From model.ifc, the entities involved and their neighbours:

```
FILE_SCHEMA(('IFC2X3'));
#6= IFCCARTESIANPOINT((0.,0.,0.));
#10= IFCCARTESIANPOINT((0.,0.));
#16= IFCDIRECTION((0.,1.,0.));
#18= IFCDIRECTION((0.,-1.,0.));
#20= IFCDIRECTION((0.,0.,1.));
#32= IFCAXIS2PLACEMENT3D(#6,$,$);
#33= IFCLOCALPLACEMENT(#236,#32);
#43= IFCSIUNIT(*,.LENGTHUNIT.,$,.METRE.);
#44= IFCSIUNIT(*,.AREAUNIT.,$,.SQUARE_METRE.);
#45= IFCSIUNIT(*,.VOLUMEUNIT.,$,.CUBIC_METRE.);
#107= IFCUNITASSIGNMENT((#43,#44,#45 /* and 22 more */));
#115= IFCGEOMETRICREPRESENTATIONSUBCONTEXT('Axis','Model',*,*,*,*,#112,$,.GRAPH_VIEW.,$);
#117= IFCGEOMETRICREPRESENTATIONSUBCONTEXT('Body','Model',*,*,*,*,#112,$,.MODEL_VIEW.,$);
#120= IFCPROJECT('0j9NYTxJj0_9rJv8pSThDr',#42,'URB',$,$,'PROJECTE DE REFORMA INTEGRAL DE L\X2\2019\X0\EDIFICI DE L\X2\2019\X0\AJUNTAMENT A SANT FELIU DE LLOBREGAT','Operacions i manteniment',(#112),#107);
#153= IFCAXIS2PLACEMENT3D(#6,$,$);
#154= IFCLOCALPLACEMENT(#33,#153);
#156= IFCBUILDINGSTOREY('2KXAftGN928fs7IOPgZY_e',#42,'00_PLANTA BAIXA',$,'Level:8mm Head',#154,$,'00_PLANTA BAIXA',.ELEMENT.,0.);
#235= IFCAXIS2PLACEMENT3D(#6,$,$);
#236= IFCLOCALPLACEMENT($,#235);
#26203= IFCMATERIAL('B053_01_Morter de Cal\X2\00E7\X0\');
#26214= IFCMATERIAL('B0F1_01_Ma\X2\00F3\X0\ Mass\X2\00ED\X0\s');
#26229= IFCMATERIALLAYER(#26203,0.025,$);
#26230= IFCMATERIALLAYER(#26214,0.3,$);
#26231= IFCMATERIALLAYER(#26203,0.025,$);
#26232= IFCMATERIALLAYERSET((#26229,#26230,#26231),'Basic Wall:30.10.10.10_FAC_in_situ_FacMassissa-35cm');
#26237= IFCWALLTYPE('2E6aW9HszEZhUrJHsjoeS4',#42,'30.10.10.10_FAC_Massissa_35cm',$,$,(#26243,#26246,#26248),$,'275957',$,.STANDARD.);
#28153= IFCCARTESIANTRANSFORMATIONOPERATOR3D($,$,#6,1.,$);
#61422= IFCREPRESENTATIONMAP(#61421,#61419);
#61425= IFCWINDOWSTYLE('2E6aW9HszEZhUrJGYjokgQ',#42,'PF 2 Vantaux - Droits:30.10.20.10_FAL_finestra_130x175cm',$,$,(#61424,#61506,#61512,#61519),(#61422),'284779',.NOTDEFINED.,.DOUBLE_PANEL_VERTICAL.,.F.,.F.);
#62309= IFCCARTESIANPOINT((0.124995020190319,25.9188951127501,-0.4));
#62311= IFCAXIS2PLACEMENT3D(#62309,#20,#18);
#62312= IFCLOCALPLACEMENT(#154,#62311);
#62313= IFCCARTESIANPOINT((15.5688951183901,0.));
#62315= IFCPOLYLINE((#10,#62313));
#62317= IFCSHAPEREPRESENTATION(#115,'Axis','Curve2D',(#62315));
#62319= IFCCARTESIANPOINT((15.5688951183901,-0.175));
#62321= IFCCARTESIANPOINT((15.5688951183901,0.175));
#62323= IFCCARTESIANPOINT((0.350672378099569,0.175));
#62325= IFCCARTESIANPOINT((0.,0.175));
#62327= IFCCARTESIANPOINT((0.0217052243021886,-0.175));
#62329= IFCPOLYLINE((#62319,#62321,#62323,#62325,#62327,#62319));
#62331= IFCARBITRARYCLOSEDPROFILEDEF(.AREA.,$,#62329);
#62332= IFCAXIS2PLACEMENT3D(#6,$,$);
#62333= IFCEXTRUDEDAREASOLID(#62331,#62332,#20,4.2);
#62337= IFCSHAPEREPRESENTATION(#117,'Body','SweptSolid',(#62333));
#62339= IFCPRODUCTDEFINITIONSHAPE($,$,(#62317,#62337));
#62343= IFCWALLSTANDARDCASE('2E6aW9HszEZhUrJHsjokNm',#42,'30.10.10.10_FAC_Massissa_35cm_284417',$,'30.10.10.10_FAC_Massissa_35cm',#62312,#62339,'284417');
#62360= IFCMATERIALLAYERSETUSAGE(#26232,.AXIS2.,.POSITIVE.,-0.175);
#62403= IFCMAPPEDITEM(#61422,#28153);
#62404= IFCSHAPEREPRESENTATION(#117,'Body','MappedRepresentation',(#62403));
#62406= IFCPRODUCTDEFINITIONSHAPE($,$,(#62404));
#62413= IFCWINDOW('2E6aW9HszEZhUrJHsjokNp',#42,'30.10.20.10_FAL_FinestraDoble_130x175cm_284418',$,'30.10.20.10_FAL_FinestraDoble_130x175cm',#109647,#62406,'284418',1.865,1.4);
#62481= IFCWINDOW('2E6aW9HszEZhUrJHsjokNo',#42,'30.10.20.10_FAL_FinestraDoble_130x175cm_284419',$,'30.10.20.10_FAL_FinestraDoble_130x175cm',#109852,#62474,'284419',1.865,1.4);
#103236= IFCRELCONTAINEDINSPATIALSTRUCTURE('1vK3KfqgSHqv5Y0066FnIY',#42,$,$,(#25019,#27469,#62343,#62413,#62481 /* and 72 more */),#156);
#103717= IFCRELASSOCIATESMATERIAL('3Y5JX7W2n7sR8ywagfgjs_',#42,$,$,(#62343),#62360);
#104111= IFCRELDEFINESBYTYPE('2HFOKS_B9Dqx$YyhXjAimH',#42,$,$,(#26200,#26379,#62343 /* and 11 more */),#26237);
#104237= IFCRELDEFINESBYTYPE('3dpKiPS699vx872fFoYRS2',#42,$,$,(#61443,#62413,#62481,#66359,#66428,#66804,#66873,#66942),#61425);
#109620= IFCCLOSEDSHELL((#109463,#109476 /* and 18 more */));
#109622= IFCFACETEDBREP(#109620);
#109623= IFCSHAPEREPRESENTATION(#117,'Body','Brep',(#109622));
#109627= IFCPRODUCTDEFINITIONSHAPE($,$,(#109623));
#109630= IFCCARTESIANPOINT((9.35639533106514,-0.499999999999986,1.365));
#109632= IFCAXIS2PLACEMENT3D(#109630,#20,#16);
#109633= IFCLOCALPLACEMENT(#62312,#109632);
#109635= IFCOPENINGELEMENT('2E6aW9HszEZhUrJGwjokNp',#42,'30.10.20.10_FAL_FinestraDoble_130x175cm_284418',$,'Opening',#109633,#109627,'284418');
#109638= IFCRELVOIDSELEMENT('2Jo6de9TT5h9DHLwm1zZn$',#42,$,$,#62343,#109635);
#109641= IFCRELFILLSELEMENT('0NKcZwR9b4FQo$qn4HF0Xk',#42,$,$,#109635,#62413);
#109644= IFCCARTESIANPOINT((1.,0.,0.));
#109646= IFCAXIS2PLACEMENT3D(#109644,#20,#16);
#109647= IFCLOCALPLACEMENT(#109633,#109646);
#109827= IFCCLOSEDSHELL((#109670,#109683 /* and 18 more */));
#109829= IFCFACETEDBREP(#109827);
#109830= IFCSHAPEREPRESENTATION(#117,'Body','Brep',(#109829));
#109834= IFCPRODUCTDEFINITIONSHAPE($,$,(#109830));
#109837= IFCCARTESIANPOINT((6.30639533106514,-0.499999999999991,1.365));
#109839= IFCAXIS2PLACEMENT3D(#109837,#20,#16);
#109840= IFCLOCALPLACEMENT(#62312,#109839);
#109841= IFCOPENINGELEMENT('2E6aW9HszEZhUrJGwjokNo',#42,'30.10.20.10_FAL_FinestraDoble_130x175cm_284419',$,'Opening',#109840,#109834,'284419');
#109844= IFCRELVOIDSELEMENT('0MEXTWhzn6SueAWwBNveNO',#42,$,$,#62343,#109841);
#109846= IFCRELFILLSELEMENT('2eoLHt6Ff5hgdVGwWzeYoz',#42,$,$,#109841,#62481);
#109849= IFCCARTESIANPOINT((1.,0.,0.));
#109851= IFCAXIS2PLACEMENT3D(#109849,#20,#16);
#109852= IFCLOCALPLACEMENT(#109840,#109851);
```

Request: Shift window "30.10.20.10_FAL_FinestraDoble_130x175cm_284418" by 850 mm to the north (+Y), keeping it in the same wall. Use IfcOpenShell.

```python
import ifcopenshell
import ifcopenshell.api.geometry
import ifcopenshell.util.placement
import ifcopenshell.util.unit

model = ifcopenshell.open("model.ifc")
unit_scale = ifcopenshell.util.unit.calculate_unit_scale(model)

window = model.by_guid("2E6aW9HszEZhUrJHsjokNp")
opening = window.FillsVoids[0].RelatingOpeningElement
wall = opening.VoidsElements[0].RelatingBuildingElement

wall_matrix = ifcopenshell.util.placement.get_local_placement(wall.ObjectPlacement)
shift = wall_matrix[:3, 0] * -0.85 / unit_scale
before = ifcopenshell.util.placement.get_local_placement(window.ObjectPlacement)[:3, 3].copy()

# The window is placed relative to its opening, so it follows when the opening moves.
matrix = ifcopenshell.util.placement.get_local_placement(opening.ObjectPlacement)
matrix[:3, 3] += shift
ifcopenshell.api.geometry.edit_object_placement(
    model, product=opening, matrix=matrix, is_si=False, should_transform_children=True
)

after = ifcopenshell.util.placement.get_local_placement(window.ObjectPlacement)[:3, 3]
print("window moved by", (after - before).round(3) + 0.0)

model.write("model_updated.ifc")
```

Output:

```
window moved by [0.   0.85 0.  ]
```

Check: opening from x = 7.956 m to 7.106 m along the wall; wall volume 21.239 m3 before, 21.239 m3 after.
